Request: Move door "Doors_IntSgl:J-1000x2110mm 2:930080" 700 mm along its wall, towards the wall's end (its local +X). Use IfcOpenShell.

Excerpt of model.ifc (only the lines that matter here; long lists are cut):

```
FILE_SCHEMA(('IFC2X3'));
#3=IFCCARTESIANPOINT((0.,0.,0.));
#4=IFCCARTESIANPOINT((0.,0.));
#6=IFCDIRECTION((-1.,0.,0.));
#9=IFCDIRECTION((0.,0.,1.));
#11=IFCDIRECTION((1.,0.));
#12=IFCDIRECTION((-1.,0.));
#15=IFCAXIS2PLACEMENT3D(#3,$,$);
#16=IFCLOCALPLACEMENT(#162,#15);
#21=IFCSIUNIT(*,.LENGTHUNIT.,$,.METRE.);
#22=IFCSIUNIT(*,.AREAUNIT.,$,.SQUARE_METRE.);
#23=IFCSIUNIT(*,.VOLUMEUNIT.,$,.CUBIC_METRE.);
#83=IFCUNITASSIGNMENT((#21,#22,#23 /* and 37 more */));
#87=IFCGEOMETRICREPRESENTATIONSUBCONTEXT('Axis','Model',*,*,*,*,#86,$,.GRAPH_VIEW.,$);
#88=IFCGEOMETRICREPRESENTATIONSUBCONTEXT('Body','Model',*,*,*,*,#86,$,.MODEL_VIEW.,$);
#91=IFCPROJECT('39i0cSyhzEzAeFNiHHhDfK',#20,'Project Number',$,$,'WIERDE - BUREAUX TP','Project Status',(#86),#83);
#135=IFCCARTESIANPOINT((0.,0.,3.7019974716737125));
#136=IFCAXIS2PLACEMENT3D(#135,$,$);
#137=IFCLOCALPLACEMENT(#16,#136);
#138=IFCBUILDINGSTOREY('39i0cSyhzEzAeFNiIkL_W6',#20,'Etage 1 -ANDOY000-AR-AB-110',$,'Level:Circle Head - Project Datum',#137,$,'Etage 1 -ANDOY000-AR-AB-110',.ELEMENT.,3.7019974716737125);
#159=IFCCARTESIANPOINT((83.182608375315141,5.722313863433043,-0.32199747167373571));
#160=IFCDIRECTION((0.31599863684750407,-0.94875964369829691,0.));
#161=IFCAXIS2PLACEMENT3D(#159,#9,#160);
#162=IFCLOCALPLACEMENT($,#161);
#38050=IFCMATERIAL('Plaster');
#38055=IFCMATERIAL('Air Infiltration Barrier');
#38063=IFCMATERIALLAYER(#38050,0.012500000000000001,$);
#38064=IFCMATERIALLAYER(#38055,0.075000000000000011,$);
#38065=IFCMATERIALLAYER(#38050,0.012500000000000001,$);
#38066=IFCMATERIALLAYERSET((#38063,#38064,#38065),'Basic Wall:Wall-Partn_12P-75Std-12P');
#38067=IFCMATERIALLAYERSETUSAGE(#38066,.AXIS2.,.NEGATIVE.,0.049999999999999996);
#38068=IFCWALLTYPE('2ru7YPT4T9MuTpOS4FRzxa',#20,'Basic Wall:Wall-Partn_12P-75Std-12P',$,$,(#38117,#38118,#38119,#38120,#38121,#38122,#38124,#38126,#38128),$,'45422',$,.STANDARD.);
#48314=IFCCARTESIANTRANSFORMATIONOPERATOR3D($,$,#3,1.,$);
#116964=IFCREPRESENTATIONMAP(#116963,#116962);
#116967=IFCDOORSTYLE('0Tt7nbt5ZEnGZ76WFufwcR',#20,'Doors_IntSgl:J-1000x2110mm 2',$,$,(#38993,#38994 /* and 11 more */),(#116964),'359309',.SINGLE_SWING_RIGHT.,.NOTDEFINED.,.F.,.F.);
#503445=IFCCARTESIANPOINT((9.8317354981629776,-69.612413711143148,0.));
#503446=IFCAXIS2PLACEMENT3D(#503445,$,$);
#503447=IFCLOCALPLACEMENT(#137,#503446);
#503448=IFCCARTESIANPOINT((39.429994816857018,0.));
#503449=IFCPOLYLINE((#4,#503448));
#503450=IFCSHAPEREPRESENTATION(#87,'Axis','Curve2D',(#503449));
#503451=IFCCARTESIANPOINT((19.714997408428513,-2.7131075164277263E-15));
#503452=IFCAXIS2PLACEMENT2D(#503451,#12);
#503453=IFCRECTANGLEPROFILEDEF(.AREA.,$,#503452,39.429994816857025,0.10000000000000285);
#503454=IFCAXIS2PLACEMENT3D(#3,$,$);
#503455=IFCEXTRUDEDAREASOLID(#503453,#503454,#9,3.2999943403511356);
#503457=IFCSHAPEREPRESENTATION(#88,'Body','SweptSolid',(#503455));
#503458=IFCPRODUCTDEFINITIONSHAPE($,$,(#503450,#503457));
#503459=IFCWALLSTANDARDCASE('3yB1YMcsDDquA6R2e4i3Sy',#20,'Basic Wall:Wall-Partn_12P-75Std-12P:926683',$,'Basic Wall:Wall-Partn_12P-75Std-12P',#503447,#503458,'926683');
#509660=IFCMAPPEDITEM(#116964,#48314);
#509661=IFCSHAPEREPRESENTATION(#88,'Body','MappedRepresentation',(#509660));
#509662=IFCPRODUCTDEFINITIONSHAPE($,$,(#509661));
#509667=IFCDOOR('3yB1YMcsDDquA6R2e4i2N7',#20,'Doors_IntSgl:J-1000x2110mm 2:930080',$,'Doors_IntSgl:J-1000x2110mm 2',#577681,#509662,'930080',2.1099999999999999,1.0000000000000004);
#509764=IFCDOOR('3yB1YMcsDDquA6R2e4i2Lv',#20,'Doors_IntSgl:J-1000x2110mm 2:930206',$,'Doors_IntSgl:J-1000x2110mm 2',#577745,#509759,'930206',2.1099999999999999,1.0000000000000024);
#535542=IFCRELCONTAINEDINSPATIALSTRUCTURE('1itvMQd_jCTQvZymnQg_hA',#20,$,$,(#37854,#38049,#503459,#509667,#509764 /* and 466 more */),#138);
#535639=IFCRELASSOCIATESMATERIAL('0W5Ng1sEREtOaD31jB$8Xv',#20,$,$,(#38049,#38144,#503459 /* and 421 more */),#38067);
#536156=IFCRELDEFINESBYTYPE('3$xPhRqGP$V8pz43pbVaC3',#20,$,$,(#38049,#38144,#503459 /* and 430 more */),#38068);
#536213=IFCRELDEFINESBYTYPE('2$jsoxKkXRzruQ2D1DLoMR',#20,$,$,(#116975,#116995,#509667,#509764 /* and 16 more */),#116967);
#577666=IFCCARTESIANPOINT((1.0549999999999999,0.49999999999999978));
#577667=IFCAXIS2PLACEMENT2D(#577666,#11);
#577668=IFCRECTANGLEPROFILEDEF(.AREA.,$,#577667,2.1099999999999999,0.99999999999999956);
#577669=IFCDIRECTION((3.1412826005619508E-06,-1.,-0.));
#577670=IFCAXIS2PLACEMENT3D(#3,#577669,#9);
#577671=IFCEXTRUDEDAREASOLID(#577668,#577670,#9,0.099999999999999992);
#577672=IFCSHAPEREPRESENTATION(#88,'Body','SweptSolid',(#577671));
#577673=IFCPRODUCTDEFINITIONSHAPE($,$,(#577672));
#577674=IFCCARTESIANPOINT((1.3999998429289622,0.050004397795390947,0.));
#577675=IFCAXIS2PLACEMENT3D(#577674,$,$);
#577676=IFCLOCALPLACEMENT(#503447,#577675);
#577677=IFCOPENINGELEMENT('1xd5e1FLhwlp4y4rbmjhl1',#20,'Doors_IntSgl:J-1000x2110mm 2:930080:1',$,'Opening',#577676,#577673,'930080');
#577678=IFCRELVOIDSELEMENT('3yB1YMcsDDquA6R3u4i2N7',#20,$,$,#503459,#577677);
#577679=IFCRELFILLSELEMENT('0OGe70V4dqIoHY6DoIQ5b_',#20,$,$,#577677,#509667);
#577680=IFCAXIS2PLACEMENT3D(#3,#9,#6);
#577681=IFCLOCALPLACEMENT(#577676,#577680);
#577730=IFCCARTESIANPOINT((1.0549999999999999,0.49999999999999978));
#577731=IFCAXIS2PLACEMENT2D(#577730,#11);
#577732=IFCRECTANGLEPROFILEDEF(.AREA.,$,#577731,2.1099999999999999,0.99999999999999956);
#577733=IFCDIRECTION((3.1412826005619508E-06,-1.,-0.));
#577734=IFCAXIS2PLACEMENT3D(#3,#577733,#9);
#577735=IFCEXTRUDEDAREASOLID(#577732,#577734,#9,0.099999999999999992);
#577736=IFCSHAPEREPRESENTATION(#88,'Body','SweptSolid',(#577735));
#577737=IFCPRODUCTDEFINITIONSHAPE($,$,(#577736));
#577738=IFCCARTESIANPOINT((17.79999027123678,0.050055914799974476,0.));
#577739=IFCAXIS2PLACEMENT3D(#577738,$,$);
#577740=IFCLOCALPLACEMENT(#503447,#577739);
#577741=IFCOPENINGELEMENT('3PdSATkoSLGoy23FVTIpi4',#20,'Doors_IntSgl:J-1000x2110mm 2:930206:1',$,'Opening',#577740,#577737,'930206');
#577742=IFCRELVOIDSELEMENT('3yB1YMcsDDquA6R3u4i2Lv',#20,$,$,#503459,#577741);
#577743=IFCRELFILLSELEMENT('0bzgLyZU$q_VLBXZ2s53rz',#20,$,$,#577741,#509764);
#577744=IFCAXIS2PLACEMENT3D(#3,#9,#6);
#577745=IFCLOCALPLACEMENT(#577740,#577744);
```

```python
import ifcopenshell
import ifcopenshell.api.geometry
import ifcopenshell.util.placement
import ifcopenshell.util.unit

model = ifcopenshell.open("model.ifc")
unit_scale = ifcopenshell.util.unit.calculate_unit_scale(model)

door = model.by_guid("3yB1YMcsDDquA6R2e4i2N7")
opening = door.FillsVoids[0].RelatingOpeningElement
wall = opening.VoidsElements[0].RelatingBuildingElement

wall_matrix = ifcopenshell.util.placement.get_local_placement(wall.ObjectPlacement)
shift = wall_matrix[:3, 0] * 0.7 / unit_scale
before = ifcopenshell.util.placement.get_local_placement(door.ObjectPlacement)[:3, 3].copy()

# The door is placed relative to its opening, so it follows when the opening moves.
matrix = ifcopenshell.util.placement.get_local_placement(opening.ObjectPlacement)
matrix[:3, 3] += shift
ifcopenshell.api.geometry.edit_object_placement(
    model, product=opening, matrix=matrix, is_si=False, should_transform_children=True
)

after = ifcopenshell.util.placement.get_local_placement(door.ObjectPlacement)[:3, 3]
print("door moved by", (after - before).round(3) + 0.0)

model.write("model-out.ifc")
```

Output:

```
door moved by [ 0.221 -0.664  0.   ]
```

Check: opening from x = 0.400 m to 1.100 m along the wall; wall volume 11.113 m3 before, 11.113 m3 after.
